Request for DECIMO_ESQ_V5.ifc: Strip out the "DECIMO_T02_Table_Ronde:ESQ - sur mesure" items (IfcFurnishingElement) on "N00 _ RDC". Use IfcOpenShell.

First a look at what the model holds.

```python
import ifcopenshell
import ifcopenshell.util.element

model = ifcopenshell.open("DECIMO_ESQ_V5.ifc")
print(model.schema)
storey = next(s for s in model.by_type("IfcBuildingStorey") if s.Name == "N00 _ RDC")
furniture = [e for e in ifcopenshell.util.element.get_decomposition(storey) if e.is_a("IfcFurnishingElement")]
seen = {}
for e in furniture:
    element_type = ifcopenshell.util.element.get_type(e)
    name = element_type.Name if element_type not in (None, e) else None
    seen[name] = seen.get(name, 0) + 1
for name, count in sorted(seen.items(), key=str):
    print(count, "x", name)
```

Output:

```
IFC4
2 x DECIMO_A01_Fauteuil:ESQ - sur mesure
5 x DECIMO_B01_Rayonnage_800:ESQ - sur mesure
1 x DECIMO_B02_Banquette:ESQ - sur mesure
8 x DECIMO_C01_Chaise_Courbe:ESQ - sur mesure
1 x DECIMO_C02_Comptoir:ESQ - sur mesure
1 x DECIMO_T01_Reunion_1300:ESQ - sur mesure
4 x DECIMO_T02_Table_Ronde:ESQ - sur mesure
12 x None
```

```python
import ifcopenshell
import ifcopenshell.api.root
import ifcopenshell.util.element

model = ifcopenshell.open("DECIMO_ESQ_V5.ifc")

storey = next(s for s in model.by_type("IfcBuildingStorey") if s.Name == "N00 _ RDC")
furniture = [e for e in ifcopenshell.util.element.get_decomposition(storey) if e.is_a("IfcFurnishingElement")]
targets = [e for e in furniture if (t := ifcopenshell.util.element.get_type(e)) not in (None, e) and t.Name == "DECIMO_T02_Table_Ronde:ESQ - sur mesure"]

for e in targets:
    ifcopenshell.api.root.remove_product(model, product=e)
print(len(targets), "removed")

model.write("DECIMO_ESQ_V5_updated.ifc")
```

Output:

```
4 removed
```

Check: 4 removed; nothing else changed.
